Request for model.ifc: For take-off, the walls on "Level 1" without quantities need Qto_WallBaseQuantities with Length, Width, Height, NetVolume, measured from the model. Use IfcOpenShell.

First a look at what the model holds.

```python
import ifcopenshell
import ifcopenshell.util.element
import ifcopenshell.util.unit

model = ifcopenshell.open("model.ifc")
print(model.schema)
for unit_type in ("LENGTHUNIT", "AREAUNIT", "VOLUMEUNIT"):
    print(unit_type, ifcopenshell.util.unit.calculate_unit_scale(model, unit_type))
storey = next(s for s in model.by_type("IfcBuildingStorey") if s.Name == "Level 1")
walls = [e for e in ifcopenshell.util.element.get_decomposition(storey) if e.is_a("IfcWall")]
for e in sorted(walls, key=lambda e: e.id()):
    print(e.id(), e.is_a(), e.Name, list(ifcopenshell.util.element.get_psets(e, qtos_only=True)), sep=" | ")
```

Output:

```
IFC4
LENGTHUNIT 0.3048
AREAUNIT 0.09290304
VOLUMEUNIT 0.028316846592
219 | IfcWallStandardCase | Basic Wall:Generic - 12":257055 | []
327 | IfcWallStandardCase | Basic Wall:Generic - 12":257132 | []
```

```python
import ifcopenshell
import ifcopenshell.api.pset
import ifcopenshell.geom
import ifcopenshell.util.element
import ifcopenshell.util.shape
import ifcopenshell.util.unit

model = ifcopenshell.open("model.ifc")
unit_scale = ifcopenshell.util.unit.calculate_unit_scale(model)
volume_scale = ifcopenshell.util.unit.calculate_unit_scale(model, "VOLUMEUNIT")
settings = ifcopenshell.geom.settings()

storey = next(s for s in model.by_type("IfcBuildingStorey") if s.Name == "Level 1")
walls = [e for e in ifcopenshell.util.element.get_decomposition(storey) if e.is_a("IfcWall")]

for e in sorted(walls, key=lambda e: e.id()):
    if ifcopenshell.util.element.get_psets(e, qtos_only=True, should_inherit=False):
        continue
    # Geometry comes back in metres, in the element's own axes.
    shape = ifcopenshell.geom.create_shape(settings, e)
    values = {
        "Length": ifcopenshell.util.shape.get_x(shape.geometry) / unit_scale,
        "Width": ifcopenshell.util.shape.get_y(shape.geometry) / unit_scale,
        "Height": ifcopenshell.util.shape.get_z(shape.geometry) / unit_scale,
        "NetVolume": ifcopenshell.util.shape.get_volume(shape.geometry) / volume_scale,
    }
    qto = ifcopenshell.api.pset.add_qto(model, product=e, name="Qto_WallBaseQuantities")
    ifcopenshell.api.pset.edit_qto(model, qto=qto, properties=values)
    print(e.id(), {k: round(v, 3) for k, v in values.items()})

model.write("model_updated.ifc")
```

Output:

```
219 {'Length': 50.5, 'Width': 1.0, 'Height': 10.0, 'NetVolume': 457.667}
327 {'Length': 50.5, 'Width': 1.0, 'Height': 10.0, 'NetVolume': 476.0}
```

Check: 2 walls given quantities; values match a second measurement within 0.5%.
